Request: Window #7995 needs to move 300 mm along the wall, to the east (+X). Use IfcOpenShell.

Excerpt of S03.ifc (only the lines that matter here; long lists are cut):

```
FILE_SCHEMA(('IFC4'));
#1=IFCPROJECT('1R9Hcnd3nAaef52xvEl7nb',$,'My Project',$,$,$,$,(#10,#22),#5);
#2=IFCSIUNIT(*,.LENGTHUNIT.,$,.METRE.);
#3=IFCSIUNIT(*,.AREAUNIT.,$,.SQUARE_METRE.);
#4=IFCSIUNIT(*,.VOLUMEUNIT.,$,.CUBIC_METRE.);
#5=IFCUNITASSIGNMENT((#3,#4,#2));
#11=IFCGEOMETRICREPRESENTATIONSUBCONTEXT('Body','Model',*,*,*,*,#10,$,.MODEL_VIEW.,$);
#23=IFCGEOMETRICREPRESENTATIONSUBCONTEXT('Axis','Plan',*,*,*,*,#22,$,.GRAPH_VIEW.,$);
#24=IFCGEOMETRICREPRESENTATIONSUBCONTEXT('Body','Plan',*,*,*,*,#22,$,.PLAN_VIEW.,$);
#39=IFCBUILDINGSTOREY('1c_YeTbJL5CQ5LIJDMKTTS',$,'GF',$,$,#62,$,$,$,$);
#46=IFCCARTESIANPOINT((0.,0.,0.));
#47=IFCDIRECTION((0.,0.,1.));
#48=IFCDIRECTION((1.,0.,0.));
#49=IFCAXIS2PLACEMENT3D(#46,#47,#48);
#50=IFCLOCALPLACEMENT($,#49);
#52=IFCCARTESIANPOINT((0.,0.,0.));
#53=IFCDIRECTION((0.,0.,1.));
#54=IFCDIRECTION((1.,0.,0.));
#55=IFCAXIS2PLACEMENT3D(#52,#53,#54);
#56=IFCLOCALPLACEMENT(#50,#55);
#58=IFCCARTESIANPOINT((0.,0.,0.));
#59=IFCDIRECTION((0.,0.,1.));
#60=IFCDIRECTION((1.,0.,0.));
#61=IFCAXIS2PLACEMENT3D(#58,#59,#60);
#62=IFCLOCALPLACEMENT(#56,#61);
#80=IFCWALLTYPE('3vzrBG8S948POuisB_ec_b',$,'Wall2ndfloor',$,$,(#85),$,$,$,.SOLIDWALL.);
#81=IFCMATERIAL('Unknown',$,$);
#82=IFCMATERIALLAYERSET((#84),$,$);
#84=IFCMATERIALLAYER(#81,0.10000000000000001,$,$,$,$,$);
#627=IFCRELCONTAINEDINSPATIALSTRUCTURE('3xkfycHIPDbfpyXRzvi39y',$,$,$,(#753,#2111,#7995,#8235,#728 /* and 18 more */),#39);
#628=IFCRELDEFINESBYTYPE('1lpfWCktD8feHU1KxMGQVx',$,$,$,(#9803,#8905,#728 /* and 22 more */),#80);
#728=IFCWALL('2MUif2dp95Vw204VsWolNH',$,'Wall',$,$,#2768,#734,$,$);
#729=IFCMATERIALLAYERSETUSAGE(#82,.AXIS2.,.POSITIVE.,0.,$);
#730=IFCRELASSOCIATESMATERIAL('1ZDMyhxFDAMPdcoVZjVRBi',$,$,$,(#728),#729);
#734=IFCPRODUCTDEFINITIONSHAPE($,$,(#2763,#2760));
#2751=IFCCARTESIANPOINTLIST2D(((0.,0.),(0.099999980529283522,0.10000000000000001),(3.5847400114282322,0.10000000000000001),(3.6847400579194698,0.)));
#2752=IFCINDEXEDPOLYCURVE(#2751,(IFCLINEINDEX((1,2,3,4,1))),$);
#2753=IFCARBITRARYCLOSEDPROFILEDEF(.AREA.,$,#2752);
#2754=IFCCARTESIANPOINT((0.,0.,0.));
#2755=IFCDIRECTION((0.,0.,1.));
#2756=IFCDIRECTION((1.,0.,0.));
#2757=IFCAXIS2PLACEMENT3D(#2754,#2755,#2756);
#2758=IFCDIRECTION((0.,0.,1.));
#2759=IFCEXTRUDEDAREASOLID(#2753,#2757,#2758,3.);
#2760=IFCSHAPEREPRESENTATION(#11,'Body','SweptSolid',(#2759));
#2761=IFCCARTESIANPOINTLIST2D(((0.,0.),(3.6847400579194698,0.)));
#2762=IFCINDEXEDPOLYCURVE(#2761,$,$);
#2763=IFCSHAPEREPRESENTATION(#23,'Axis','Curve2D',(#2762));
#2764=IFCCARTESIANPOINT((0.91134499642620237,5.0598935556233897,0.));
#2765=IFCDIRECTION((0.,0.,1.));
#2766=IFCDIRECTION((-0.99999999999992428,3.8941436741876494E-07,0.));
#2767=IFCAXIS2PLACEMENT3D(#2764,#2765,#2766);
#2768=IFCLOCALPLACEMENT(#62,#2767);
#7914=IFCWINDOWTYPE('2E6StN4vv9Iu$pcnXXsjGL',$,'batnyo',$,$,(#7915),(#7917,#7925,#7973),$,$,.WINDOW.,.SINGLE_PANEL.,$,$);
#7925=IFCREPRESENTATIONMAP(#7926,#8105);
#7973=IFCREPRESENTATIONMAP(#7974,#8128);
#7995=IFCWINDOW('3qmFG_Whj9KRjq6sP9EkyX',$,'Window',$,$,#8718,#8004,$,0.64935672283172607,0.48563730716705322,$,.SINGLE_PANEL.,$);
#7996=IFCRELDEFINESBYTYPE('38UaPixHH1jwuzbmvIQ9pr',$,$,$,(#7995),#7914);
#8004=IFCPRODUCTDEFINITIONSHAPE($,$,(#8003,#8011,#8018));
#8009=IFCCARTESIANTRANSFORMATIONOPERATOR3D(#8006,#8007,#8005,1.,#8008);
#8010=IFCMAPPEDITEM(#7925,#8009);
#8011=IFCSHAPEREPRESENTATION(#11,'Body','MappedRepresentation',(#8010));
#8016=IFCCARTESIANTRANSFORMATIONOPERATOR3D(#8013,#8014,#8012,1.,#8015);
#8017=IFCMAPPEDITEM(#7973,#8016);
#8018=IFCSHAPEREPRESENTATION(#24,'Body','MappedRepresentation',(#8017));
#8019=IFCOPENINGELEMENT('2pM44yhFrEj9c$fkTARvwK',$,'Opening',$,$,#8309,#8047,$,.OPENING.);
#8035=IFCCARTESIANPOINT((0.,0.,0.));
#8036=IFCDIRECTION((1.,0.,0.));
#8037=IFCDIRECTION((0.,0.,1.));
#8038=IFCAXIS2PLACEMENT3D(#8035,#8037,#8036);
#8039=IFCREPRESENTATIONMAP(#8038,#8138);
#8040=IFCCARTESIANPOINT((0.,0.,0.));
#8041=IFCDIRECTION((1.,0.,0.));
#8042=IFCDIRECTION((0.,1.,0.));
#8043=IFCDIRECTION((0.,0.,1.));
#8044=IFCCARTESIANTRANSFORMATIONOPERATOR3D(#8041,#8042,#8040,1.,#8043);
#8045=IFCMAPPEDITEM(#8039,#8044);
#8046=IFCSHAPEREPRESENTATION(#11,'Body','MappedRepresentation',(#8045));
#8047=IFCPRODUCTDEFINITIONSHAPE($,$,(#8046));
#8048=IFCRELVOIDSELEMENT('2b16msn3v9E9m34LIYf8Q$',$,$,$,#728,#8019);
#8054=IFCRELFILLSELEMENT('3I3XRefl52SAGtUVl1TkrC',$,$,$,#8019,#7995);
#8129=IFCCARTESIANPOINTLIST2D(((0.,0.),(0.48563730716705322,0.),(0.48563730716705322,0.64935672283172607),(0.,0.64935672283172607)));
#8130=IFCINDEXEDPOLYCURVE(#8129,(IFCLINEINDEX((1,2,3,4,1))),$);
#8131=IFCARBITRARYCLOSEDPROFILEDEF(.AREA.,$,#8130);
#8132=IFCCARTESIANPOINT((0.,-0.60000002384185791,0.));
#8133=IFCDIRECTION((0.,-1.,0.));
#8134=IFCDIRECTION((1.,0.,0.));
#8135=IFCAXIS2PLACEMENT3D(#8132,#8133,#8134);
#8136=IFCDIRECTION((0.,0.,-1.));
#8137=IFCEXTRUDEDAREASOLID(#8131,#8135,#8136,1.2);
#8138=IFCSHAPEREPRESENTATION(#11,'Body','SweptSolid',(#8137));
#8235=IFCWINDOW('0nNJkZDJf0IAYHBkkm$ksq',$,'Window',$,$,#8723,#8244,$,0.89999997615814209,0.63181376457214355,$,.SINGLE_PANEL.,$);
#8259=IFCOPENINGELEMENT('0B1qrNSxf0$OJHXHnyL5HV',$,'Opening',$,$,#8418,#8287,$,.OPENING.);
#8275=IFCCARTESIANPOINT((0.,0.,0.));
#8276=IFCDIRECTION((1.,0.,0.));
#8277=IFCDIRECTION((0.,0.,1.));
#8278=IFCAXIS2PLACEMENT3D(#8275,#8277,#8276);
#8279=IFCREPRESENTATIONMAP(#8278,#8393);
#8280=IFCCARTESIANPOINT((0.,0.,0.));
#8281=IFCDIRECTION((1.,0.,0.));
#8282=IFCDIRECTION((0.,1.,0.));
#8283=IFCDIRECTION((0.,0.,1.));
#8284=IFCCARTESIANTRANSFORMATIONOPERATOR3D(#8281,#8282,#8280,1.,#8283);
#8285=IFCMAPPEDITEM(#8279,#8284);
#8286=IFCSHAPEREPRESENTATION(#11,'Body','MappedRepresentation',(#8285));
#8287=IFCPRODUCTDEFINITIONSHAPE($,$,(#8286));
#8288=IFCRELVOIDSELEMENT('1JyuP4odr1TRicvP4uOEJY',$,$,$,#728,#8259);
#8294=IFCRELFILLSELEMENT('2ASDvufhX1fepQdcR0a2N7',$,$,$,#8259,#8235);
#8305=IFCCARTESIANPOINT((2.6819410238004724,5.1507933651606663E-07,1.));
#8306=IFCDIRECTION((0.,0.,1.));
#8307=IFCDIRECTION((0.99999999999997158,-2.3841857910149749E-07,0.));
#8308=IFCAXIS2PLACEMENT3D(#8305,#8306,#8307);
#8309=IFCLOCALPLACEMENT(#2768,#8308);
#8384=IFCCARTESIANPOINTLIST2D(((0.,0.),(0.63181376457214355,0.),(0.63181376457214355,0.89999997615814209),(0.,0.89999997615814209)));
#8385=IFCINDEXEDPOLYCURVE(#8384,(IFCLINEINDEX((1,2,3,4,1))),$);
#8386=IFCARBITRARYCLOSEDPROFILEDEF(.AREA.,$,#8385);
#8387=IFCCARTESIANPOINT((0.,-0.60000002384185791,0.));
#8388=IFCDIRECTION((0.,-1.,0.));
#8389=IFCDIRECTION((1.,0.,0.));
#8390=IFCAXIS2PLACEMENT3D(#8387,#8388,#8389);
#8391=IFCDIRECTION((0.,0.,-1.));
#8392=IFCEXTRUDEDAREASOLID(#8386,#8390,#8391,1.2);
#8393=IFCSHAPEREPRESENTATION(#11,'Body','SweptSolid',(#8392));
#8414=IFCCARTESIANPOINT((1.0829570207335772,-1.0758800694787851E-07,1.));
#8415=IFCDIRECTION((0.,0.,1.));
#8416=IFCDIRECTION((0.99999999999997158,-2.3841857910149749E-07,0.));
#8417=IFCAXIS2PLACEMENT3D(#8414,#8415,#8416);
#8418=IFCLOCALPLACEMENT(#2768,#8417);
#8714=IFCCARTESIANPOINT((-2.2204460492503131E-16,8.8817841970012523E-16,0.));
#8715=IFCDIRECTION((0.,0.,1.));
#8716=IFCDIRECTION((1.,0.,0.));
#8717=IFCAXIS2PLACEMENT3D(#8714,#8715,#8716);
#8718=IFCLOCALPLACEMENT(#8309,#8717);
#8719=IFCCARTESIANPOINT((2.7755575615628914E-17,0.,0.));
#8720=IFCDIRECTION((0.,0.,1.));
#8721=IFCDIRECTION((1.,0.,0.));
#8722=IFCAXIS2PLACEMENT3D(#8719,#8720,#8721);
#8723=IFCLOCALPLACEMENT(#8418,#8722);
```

```python
import ifcopenshell
import ifcopenshell.api.geometry
import ifcopenshell.util.placement
import ifcopenshell.util.unit

model = ifcopenshell.open("S03.ifc")
unit_scale = ifcopenshell.util.unit.calculate_unit_scale(model)

window = model.by_id(7995)
opening = window.FillsVoids[0].RelatingOpeningElement
wall = opening.VoidsElements[0].RelatingBuildingElement

wall_matrix = ifcopenshell.util.placement.get_local_placement(wall.ObjectPlacement)
shift = wall_matrix[:3, 0] * -0.3 / unit_scale
before = ifcopenshell.util.placement.get_local_placement(window.ObjectPlacement)[:3, 3].copy()

# The window is placed relative to its opening, so it follows when the opening moves.
matrix = ifcopenshell.util.placement.get_local_placement(opening.ObjectPlacement)
matrix[:3, 3] += shift
ifcopenshell.api.geometry.edit_object_placement(
    model, product=opening, matrix=matrix, is_si=False, should_transform_children=True
)

after = ifcopenshell.util.placement.get_local_placement(window.ObjectPlacement)[:3, 3]
print("window moved by", (after - before).round(3) + 0.0)

model.write("S03-out.ifc")
```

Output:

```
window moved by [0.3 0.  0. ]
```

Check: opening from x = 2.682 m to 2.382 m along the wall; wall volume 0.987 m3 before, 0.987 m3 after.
